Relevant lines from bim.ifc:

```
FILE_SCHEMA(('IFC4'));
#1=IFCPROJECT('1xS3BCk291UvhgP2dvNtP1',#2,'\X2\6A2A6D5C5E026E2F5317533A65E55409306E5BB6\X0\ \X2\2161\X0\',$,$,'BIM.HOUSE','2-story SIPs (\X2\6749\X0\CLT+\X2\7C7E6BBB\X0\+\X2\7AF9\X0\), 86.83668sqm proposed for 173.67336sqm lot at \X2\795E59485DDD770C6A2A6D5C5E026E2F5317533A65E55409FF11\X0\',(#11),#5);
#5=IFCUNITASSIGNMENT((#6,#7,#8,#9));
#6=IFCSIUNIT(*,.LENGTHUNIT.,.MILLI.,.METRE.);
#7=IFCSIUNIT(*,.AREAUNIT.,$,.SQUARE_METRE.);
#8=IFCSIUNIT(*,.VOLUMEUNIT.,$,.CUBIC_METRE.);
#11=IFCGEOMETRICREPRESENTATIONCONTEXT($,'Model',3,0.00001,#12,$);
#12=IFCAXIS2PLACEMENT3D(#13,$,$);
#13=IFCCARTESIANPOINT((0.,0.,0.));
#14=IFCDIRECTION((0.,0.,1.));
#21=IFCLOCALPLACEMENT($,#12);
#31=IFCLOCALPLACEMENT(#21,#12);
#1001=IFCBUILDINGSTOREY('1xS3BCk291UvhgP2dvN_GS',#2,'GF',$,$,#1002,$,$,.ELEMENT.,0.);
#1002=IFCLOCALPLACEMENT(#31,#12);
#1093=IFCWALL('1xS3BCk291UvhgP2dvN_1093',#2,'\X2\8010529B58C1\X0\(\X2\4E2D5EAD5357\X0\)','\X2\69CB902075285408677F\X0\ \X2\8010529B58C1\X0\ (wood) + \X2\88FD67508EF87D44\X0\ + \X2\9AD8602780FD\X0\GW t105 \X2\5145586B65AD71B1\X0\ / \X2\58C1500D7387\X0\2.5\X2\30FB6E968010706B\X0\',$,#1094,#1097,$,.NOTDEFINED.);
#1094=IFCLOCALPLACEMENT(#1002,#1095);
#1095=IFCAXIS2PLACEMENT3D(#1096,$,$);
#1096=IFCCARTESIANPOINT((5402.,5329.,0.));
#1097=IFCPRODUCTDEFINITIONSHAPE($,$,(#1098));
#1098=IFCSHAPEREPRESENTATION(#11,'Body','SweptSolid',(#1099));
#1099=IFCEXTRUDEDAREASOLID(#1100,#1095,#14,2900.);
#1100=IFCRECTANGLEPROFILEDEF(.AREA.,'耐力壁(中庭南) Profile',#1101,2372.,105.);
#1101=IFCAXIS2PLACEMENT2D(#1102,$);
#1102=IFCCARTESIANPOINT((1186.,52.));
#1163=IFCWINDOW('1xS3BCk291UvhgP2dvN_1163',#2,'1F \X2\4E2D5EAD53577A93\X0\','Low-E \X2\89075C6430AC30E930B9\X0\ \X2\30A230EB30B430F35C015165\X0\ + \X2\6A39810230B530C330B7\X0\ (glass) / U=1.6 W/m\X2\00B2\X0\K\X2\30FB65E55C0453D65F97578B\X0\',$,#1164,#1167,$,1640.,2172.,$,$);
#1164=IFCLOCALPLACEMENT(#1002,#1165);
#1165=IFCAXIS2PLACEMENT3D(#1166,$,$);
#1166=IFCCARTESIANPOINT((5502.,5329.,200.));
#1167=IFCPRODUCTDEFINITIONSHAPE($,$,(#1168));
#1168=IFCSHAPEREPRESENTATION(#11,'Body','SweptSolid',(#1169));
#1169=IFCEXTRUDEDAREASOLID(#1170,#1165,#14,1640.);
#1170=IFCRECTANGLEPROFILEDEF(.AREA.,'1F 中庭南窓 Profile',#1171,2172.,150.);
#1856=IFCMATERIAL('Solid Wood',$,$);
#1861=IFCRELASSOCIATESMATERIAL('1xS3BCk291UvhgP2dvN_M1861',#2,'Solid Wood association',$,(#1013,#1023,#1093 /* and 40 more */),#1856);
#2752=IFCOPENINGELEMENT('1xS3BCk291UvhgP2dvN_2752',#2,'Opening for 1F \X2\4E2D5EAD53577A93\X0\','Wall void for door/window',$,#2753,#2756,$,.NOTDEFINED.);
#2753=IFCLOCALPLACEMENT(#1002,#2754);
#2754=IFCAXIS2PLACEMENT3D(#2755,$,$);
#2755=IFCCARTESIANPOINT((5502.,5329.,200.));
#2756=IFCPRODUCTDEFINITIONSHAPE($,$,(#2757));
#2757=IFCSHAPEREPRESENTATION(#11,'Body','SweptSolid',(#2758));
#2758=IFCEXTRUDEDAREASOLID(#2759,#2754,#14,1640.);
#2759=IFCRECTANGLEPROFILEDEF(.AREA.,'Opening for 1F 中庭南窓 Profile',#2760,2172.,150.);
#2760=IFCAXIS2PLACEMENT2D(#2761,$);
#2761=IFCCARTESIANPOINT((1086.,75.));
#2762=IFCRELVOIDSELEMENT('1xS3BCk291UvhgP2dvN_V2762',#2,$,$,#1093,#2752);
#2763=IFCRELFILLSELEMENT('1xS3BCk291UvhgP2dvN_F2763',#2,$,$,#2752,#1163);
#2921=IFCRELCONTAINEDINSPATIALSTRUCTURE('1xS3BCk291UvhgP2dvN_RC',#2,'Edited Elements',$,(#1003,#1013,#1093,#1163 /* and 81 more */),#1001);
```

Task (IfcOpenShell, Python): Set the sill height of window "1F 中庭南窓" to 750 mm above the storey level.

```python
import numpy as np
import ifcopenshell
import ifcopenshell.api.geometry
import ifcopenshell.geom
import ifcopenshell.util.element
import ifcopenshell.util.placement
import ifcopenshell.util.shape
import ifcopenshell.util.unit

model = ifcopenshell.open("bim.ifc")
unit_scale = ifcopenshell.util.unit.calculate_unit_scale(model)

window = model.by_guid("1xS3BCk291UvhgP2dvN_1163")
opening = window.FillsVoids[0].RelatingOpeningElement
storey = ifcopenshell.util.element.get_container(window, ifc_class="IfcBuildingStorey")
level = ifcopenshell.util.placement.get_local_placement(storey.ObjectPlacement)[2, 3]

# The opening's origin need not be at the sill, so measure its lowest point.
shape = ifcopenshell.geom.create_shape(ifcopenshell.geom.settings(), opening)
bottom = ifcopenshell.util.shape.get_shape_bottom_elevation(shape, shape.geometry) / unit_scale
dz = level + 0.75 / unit_scale - bottom

shift = np.array([0.0, 0.0, dz])
# The window is not placed relative to its opening, so move both.
for product in (opening, window):
    matrix = ifcopenshell.util.placement.get_local_placement(product.ObjectPlacement)
    matrix[:3, 3] += shift
    ifcopenshell.api.geometry.edit_object_placement(model, product=product, matrix=matrix, is_si=False)

print(f"moved by {dz * unit_scale:+.3f} m")

model.write("bim_rev.ifc")
```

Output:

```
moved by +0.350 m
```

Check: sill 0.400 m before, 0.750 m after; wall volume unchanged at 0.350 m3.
